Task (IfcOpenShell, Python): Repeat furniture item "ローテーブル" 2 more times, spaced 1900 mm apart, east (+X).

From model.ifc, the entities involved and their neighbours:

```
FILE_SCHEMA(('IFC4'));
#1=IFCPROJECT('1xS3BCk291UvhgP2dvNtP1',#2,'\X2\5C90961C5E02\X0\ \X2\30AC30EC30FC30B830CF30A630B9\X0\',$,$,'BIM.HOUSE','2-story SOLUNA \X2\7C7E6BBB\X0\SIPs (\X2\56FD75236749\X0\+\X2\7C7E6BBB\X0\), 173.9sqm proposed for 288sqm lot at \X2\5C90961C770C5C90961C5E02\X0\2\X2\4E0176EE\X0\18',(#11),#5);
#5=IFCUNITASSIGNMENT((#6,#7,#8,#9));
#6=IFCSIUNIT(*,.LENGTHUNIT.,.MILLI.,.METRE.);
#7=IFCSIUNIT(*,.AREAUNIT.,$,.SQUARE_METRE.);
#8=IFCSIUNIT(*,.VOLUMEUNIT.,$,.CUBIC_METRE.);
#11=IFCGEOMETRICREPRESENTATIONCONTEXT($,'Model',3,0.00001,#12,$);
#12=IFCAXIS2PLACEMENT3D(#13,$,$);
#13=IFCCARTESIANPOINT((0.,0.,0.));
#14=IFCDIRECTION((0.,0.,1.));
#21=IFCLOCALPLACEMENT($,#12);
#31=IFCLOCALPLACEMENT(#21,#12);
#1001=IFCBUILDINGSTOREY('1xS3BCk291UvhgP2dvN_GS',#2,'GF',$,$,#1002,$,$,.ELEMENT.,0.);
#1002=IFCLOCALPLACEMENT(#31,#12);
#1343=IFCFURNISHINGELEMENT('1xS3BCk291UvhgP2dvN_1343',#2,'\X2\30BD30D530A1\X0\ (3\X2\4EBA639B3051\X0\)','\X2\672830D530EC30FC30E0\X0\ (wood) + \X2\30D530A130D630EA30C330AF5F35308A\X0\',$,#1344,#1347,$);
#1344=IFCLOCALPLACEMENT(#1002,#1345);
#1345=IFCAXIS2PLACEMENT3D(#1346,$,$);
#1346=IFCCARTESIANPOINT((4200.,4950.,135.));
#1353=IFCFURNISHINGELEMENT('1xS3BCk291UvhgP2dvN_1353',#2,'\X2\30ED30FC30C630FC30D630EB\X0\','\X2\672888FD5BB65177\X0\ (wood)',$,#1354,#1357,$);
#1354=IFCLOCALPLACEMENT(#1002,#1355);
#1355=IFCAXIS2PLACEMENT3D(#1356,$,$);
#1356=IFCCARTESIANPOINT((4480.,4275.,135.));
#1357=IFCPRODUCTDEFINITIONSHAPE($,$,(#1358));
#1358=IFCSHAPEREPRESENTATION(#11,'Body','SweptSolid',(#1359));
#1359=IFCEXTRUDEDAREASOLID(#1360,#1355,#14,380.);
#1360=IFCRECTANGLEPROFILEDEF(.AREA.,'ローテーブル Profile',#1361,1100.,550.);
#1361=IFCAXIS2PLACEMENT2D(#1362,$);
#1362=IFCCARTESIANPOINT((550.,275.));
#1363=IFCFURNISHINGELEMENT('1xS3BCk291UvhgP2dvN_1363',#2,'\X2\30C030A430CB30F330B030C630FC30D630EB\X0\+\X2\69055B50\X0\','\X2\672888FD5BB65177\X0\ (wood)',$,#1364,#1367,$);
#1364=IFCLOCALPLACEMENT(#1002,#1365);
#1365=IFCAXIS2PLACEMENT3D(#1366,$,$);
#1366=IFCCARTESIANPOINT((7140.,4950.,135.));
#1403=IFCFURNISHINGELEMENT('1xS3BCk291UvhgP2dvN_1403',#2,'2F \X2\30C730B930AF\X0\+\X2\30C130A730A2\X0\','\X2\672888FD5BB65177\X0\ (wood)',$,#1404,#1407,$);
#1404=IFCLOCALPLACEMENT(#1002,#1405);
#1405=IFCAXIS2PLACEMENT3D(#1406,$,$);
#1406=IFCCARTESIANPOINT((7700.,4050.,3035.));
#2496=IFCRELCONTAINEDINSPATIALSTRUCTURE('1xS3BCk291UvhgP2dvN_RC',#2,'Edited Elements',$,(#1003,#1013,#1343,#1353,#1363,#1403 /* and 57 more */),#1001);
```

```python
import numpy as np
import ifcopenshell
import ifcopenshell.api.geometry
import ifcopenshell.api.root
import ifcopenshell.util.element
import ifcopenshell.util.placement
import ifcopenshell.util.unit

model = ifcopenshell.open("model.ifc")
unit_scale = ifcopenshell.util.unit.calculate_unit_scale(model)


def reuse_history(source, copy):
    """copy_class also copies each property set's owner history, people and application; keep the originals."""
    for rel in copy.IsDefinedBy:
        if rel.is_a("IfcRelDefinesByProperties") and (history := rel.RelatingPropertyDefinition.OwnerHistory):
            rel.RelatingPropertyDefinition.OwnerHistory = source.OwnerHistory
            ifcopenshell.util.element.remove_deep2(model, history)


source = model.by_guid("1xS3BCk291UvhgP2dvN_1353")
base = ifcopenshell.util.placement.get_local_placement(source.ObjectPlacement)
step = np.array([1.0, 0.0, 0.0]) * 1.9 / unit_scale

for i in range(1, 3):
    copy = ifcopenshell.api.root.copy_class(model, product=source)
    copy.Representation = ifcopenshell.util.element.copy_deep(
        model, source.Representation, exclude=["IfcGeometricRepresentationContext", "IfcRepresentationMap"]
    )
    reuse_history(source, copy)
    matrix = base.copy()
    matrix[:3, 3] += i * step
    print("added at", matrix[:3, 3].round(3) + 0.0)
    ifcopenshell.api.geometry.edit_object_placement(model, product=copy, matrix=matrix, is_si=False)

model.write("model-out.ifc")
```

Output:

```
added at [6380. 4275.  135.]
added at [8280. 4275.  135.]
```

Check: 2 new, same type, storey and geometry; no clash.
